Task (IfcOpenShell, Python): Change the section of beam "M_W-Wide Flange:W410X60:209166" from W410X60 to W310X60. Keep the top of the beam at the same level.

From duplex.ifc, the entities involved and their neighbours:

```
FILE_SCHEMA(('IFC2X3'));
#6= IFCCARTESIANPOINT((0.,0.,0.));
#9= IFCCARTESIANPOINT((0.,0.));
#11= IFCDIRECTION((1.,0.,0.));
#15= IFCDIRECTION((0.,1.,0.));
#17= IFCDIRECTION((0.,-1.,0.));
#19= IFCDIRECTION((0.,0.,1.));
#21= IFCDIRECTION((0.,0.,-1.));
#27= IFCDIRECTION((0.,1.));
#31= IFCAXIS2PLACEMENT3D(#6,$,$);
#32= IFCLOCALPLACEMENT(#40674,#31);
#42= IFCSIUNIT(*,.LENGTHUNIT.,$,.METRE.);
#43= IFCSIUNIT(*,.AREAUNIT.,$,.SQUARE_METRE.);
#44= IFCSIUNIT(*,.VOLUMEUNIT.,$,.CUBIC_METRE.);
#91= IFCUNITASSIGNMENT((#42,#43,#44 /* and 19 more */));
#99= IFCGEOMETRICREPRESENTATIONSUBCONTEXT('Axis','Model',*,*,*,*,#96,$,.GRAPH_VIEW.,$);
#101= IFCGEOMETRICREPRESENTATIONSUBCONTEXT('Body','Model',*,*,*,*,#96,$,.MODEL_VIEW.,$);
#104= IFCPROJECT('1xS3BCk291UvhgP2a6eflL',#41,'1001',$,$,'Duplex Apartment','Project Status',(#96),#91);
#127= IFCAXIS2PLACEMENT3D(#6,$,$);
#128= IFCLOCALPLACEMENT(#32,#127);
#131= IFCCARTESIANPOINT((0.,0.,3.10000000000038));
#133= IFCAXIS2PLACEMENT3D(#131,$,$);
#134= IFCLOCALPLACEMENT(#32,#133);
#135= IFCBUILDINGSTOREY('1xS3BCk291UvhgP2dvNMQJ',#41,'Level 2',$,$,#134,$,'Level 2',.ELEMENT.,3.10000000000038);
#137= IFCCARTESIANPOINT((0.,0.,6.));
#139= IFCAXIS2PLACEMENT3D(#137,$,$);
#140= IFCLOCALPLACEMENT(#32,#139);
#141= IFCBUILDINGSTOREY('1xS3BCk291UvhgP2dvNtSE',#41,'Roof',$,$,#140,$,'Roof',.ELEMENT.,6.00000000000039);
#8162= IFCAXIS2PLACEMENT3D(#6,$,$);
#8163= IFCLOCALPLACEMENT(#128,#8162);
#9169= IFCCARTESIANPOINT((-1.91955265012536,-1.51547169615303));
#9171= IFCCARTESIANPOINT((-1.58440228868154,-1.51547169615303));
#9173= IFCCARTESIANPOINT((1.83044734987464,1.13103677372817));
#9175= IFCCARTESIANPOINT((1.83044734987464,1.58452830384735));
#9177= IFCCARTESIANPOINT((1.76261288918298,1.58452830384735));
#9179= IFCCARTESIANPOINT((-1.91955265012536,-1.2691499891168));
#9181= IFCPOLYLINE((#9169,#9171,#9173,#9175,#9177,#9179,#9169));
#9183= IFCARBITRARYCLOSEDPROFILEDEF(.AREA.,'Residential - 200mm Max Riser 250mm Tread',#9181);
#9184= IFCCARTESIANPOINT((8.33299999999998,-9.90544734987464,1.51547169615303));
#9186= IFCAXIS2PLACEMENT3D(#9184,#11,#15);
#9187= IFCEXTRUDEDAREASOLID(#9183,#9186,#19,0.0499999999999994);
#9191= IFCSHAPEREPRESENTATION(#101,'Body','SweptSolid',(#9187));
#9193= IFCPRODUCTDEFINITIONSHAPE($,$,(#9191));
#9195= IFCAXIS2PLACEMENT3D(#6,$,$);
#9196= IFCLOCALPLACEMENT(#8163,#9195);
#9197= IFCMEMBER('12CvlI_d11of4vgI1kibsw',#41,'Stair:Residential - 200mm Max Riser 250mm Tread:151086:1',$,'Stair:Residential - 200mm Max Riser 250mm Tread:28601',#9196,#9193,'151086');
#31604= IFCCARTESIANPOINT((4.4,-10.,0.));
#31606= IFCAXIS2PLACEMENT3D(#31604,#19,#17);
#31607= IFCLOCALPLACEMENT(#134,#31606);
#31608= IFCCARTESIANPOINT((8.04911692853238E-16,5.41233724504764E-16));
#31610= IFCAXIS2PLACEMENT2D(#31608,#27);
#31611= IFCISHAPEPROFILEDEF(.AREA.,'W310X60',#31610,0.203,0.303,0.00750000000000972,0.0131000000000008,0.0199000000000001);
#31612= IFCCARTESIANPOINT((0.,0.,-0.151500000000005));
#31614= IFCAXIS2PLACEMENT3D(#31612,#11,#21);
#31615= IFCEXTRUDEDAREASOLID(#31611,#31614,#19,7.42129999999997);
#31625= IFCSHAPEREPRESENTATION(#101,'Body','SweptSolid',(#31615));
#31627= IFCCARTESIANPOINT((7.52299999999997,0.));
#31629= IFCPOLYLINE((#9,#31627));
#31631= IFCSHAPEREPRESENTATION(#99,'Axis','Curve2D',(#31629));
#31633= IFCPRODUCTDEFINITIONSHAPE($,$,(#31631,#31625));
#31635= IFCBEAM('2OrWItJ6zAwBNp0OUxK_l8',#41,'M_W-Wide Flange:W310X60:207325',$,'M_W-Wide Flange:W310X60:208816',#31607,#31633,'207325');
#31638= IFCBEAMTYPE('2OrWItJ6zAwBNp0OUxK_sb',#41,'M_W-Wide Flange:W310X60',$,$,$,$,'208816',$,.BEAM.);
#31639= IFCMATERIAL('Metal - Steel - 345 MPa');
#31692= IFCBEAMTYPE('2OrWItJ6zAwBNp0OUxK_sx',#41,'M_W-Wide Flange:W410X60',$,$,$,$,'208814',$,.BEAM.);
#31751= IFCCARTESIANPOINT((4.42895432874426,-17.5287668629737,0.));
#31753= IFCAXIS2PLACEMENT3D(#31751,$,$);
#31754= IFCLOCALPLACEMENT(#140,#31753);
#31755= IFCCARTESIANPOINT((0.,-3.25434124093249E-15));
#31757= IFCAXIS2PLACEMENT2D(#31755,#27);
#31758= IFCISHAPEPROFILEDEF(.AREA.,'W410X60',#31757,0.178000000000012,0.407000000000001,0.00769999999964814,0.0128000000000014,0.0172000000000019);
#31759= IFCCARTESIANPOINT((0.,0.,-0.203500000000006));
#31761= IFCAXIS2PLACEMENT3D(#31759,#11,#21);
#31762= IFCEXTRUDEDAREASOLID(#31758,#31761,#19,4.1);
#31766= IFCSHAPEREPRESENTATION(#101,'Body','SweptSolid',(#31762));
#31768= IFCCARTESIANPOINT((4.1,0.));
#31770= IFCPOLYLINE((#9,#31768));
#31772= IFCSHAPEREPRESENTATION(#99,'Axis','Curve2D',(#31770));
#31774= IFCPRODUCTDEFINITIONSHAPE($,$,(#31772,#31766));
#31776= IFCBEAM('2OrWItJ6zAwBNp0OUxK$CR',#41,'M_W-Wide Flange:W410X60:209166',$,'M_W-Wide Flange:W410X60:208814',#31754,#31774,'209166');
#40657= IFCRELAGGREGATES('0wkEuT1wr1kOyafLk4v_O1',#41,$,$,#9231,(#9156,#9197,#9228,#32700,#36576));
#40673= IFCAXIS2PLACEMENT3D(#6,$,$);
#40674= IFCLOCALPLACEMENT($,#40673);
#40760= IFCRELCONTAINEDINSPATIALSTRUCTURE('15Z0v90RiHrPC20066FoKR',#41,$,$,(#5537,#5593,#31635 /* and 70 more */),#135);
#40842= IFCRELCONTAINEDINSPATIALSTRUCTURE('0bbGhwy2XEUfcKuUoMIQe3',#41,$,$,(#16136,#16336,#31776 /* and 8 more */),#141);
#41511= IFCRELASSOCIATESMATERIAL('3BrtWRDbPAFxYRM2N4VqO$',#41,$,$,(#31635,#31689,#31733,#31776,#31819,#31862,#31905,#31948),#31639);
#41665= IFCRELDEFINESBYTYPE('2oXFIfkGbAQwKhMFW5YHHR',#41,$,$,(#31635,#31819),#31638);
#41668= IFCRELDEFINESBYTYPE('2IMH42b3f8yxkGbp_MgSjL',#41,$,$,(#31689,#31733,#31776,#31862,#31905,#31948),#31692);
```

```python
import ifcopenshell
import ifcopenshell.api.type
import ifcopenshell.util.element
import ifcopenshell.util.representation

model = ifcopenshell.open("duplex.ifc")

member = model.by_guid("2OrWItJ6zAwBNp0OUxK$CR")
source = next(p for p in model.by_type("IfcIShapeProfileDef") if p.ProfileName == "W310X60")

body = ifcopenshell.util.representation.get_representation(member, "Model", "Body")
solid = body.Items[0]
old_profile = solid.SweptArea

# Copy the section's sizes but keep this member's own profile position.
profile = ifcopenshell.util.element.copy(model, source)
# Profiles are centred, so shift by half the change in depth to hold the top.
shift = (old_profile.OverallDepth - profile.OverallDepth) / 2
x, y = old_profile.Position.Location.Coordinates
up = (-1.0, 0.0)  # upwards, in the solid's own plane
location = model.createIfcCartesianPoint((x + up[0] * shift, y + up[1] * shift))
profile.Position = model.createIfcAxis2Placement2D(location, old_profile.Position.RefDirection)
solid.SweptArea = profile
if not model.get_total_inverses(old_profile):
    ifcopenshell.util.element.remove_deep2(model, old_profile)

new_type = model.by_guid("2OrWItJ6zAwBNp0OUxK_sb")
ifcopenshell.api.type.assign_type(
    model, related_objects=[member], relating_type=new_type, should_map_representations=False
)
member.Name = member.Name.replace("W410X60", "W310X60")
member.ObjectType = "M_W-Wide Flange:W310X60:208814"

print(solid.SweptArea)

model.write("duplex_updated.ifc")
```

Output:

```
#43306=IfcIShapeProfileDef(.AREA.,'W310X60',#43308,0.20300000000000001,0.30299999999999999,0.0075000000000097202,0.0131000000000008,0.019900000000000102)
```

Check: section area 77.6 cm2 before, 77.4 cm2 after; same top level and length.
